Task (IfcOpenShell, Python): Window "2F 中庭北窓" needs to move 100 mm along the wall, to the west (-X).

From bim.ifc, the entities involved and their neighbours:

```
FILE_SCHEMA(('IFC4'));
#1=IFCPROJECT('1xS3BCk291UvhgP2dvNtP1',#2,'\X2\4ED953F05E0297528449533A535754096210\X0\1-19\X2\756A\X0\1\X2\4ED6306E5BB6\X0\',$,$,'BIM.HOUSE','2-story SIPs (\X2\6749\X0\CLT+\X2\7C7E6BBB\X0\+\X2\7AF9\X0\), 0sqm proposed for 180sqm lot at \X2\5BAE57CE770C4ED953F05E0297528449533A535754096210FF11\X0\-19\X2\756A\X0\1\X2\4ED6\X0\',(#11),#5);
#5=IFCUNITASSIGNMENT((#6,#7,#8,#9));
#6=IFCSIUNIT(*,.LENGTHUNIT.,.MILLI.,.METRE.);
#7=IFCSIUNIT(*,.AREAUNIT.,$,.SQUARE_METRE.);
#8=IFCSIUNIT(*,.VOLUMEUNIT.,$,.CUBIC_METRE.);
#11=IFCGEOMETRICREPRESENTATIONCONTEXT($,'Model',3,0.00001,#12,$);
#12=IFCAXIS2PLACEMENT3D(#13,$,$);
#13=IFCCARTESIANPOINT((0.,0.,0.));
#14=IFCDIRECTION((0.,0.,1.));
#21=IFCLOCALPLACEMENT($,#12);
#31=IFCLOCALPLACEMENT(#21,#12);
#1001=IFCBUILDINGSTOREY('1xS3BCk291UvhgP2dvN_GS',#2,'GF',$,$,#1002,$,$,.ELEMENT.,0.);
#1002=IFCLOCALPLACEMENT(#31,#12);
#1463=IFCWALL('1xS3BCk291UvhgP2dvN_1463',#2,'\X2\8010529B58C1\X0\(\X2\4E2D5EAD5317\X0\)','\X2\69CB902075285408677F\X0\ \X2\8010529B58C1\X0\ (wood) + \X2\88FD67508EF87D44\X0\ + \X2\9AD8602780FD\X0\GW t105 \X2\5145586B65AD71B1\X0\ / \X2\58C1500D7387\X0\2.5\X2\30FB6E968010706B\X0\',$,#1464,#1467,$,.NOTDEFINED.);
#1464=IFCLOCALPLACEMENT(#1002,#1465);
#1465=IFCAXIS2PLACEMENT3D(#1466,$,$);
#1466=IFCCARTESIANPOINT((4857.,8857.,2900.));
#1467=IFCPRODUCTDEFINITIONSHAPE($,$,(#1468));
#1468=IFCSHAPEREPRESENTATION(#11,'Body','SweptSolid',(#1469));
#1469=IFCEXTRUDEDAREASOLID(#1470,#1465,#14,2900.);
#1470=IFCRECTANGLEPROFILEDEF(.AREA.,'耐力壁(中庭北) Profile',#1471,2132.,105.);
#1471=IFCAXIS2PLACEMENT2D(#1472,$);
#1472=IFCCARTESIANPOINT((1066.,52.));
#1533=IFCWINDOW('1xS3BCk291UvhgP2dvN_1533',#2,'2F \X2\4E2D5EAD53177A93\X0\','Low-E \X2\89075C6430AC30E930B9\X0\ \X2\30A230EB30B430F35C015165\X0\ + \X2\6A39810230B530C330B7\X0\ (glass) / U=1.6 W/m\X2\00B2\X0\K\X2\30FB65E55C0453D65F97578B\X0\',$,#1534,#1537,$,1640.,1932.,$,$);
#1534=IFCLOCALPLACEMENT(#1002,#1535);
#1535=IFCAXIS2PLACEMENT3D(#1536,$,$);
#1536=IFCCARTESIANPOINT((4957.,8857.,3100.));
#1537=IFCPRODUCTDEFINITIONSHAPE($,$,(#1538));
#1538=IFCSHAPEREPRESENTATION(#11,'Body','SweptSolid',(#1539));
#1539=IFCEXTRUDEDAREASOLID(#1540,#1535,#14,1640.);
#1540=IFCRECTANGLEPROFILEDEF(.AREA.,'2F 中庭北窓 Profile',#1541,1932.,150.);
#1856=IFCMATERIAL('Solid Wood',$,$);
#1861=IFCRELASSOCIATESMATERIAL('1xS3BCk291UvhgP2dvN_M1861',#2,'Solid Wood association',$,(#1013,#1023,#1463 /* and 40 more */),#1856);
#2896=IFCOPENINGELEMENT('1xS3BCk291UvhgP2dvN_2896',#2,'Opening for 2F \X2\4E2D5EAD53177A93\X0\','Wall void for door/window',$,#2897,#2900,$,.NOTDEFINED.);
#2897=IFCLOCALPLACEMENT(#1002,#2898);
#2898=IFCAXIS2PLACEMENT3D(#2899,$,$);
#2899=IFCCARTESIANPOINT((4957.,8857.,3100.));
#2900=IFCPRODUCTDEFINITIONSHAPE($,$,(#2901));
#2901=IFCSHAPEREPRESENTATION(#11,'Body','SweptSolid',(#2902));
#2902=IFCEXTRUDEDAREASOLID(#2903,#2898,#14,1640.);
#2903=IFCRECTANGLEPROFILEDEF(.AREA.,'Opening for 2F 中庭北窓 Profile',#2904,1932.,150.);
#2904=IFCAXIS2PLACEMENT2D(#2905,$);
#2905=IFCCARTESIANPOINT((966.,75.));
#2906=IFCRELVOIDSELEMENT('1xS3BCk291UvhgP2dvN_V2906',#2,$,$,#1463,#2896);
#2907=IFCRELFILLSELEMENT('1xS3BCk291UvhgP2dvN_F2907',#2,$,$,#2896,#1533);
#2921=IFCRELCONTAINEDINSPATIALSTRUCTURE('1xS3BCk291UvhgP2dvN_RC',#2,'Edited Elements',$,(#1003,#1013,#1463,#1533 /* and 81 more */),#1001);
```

```python
import ifcopenshell
import ifcopenshell.api.geometry
import ifcopenshell.util.placement
import ifcopenshell.util.unit

model = ifcopenshell.open("bim.ifc")
unit_scale = ifcopenshell.util.unit.calculate_unit_scale(model)

window = model.by_guid("1xS3BCk291UvhgP2dvN_1533")
opening = window.FillsVoids[0].RelatingOpeningElement
wall = opening.VoidsElements[0].RelatingBuildingElement

wall_matrix = ifcopenshell.util.placement.get_local_placement(wall.ObjectPlacement)
shift = wall_matrix[:3, 0] * -0.1 / unit_scale
before = ifcopenshell.util.placement.get_local_placement(window.ObjectPlacement)[:3, 3].copy()

# The window is not placed relative to its opening, so move both.
for product in (opening, window):
    matrix = ifcopenshell.util.placement.get_local_placement(product.ObjectPlacement)
    matrix[:3, 3] += shift
    ifcopenshell.api.geometry.edit_object_placement(model, product=product, matrix=matrix, is_si=False)

after = ifcopenshell.util.placement.get_local_placement(window.ObjectPlacement)[:3, 3]
print("window moved by", (after - before).round(3) + 0.0)

model.write("bim_rev.ifc")
```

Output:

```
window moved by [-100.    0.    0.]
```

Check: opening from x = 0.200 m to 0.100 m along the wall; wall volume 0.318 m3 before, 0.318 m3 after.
